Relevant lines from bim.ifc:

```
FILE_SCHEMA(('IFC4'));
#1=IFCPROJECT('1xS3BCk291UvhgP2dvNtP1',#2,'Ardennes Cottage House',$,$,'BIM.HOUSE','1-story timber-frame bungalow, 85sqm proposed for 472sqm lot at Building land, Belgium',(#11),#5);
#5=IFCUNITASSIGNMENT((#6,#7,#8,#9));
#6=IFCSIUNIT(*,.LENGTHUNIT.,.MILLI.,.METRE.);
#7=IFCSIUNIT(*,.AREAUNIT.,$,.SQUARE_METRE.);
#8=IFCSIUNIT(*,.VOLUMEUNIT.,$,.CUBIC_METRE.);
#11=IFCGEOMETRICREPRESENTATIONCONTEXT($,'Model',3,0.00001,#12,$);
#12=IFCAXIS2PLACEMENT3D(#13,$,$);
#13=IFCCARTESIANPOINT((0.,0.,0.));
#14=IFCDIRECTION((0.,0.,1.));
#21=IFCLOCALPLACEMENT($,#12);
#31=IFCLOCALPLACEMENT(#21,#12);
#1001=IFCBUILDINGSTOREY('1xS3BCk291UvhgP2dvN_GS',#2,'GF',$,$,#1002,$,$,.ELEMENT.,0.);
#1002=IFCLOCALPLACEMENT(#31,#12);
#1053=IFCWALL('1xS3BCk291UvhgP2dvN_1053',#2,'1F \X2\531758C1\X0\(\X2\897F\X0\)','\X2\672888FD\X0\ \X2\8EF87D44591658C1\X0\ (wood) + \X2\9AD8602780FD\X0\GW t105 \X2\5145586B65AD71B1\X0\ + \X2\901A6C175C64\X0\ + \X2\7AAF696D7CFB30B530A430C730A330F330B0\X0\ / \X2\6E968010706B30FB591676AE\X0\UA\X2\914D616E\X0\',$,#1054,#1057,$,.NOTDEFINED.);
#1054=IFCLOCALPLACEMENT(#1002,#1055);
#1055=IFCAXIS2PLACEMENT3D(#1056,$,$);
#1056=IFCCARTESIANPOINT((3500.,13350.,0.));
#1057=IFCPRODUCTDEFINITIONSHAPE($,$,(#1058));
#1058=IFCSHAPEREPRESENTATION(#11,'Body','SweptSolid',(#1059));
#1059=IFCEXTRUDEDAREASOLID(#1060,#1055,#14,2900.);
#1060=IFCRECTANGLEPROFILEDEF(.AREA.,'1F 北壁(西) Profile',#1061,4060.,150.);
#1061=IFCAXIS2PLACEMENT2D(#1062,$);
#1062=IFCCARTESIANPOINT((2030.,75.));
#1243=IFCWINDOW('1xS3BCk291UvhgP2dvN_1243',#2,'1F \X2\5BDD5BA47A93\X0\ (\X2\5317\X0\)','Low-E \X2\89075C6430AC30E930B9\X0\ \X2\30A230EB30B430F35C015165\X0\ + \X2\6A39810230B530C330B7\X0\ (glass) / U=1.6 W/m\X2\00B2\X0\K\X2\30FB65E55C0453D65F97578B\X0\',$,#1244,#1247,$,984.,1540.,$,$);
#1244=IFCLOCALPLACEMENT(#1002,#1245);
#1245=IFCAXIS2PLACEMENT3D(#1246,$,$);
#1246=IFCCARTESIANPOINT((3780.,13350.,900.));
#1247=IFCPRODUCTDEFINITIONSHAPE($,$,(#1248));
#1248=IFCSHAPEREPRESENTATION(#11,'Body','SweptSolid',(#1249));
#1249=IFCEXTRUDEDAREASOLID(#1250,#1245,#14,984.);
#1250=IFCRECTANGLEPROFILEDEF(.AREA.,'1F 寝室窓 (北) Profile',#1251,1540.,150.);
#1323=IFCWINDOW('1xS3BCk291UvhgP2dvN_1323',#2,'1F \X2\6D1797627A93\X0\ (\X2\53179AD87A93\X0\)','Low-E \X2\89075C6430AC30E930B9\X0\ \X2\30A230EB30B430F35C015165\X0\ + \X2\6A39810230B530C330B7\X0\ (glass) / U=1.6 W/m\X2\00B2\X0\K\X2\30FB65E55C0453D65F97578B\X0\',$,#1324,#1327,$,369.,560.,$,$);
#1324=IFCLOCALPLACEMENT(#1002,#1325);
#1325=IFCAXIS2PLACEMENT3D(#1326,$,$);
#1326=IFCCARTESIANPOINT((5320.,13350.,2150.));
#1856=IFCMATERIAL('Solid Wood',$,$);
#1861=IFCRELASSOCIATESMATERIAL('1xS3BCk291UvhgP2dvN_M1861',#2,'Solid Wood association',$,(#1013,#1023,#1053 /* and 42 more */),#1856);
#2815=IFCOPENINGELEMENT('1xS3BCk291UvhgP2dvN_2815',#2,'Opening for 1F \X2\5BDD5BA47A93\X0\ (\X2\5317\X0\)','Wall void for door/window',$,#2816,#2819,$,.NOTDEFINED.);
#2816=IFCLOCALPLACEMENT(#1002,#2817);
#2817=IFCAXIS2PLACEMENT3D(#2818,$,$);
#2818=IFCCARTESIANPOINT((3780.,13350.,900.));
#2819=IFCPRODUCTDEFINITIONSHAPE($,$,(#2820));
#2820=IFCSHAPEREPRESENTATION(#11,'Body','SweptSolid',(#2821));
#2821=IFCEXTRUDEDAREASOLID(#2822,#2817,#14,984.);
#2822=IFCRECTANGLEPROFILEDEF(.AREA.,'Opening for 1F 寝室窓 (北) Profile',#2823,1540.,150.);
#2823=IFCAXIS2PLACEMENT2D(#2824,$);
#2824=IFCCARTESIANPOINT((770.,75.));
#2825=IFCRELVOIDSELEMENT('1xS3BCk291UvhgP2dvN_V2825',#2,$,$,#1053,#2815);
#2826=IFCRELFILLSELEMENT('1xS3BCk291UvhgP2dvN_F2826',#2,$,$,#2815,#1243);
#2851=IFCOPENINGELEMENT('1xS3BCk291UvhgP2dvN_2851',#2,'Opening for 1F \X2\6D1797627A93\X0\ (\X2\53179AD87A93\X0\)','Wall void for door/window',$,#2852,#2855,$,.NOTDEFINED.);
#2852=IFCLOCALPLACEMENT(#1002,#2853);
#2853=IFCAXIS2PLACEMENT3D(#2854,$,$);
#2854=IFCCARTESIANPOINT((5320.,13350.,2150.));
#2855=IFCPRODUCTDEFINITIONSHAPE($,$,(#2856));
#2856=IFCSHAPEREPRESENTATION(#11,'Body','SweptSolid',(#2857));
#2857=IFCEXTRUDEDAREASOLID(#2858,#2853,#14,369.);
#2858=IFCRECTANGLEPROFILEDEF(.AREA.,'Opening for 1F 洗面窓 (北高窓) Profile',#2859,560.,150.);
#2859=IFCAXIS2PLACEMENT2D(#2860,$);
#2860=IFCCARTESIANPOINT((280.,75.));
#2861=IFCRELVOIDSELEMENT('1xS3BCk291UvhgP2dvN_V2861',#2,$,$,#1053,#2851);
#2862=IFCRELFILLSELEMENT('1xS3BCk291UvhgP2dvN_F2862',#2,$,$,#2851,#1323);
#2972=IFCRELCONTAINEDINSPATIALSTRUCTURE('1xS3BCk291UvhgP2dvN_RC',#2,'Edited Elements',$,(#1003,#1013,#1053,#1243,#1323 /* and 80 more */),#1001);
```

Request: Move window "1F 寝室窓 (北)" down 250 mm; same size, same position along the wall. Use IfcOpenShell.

```python
import numpy as np
import ifcopenshell
import ifcopenshell.api.geometry
import ifcopenshell.util.placement
import ifcopenshell.util.unit

model = ifcopenshell.open("bim.ifc")
unit_scale = ifcopenshell.util.unit.calculate_unit_scale(model)

window = model.by_id(1243)
opening = window.FillsVoids[0].RelatingOpeningElement
dz = -0.25 / unit_scale

shift = np.array([0.0, 0.0, dz])
# The window is not placed relative to its opening, so move both.
for product in (opening, window):
    matrix = ifcopenshell.util.placement.get_local_placement(product.ObjectPlacement)
    matrix[:3, 3] += shift
    ifcopenshell.api.geometry.edit_object_placement(model, product=product, matrix=matrix, is_si=False)

print(f"moved by {dz * unit_scale:+.3f} m")

model.write("bim_rev.ifc")
```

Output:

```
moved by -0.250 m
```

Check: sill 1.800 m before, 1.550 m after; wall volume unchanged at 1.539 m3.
